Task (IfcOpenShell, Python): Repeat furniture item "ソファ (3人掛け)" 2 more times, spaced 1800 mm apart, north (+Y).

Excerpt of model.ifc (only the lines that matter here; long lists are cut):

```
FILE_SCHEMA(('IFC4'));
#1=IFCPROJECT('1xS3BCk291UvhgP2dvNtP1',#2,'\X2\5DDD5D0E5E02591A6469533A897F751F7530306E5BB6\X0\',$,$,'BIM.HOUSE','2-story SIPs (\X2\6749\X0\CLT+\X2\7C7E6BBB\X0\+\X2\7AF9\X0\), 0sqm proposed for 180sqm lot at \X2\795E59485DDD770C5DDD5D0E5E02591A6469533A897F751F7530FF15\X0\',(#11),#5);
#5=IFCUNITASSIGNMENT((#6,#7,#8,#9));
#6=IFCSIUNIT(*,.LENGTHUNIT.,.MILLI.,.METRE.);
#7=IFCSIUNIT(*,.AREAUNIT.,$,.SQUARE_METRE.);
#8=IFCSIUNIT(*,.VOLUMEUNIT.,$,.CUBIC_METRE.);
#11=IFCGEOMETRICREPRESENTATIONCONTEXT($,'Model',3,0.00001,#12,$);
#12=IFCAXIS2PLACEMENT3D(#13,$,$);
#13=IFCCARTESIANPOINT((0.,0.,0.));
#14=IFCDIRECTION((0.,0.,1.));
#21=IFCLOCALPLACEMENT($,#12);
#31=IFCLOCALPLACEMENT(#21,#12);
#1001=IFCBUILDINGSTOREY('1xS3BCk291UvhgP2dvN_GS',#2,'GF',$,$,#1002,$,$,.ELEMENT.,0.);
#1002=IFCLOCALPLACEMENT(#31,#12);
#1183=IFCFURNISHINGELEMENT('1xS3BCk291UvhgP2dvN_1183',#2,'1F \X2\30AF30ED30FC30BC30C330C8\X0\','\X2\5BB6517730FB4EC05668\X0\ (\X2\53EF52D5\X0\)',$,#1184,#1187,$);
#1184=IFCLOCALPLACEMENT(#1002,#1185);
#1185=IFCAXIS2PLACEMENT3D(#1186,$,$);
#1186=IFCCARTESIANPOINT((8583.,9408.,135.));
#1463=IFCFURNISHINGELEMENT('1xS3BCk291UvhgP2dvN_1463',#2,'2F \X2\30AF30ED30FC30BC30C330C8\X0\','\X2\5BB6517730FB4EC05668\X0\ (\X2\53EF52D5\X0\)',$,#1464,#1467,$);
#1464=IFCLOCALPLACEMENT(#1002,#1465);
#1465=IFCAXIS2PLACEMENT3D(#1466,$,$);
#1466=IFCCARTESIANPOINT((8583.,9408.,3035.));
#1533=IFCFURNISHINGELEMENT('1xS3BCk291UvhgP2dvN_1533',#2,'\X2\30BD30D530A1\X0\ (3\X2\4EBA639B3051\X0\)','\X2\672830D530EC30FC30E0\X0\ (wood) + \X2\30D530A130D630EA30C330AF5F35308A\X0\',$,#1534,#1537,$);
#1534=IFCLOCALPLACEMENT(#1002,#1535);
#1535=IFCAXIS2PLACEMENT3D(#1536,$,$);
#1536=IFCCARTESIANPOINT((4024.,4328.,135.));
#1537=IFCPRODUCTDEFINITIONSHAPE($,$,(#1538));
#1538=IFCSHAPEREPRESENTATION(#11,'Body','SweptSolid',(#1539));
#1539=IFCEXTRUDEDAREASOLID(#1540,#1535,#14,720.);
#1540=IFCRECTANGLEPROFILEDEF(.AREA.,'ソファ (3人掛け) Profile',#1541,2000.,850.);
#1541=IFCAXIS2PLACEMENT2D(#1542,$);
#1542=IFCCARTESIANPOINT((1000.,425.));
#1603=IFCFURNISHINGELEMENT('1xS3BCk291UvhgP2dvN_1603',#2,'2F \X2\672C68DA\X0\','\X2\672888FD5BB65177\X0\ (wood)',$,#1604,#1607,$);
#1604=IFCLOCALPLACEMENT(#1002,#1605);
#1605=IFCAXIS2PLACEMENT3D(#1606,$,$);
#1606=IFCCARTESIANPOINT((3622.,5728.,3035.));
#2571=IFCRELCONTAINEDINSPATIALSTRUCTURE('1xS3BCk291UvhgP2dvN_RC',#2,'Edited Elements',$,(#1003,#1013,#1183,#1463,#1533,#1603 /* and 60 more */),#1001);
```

```python
import numpy as np
import ifcopenshell
import ifcopenshell.api.geometry
import ifcopenshell.api.root
import ifcopenshell.util.element
import ifcopenshell.util.placement
import ifcopenshell.util.unit

model = ifcopenshell.open("model.ifc")
unit_scale = ifcopenshell.util.unit.calculate_unit_scale(model)


def reuse_history(source, copy):
    """copy_class also copies each property set's owner history, people and application; keep the originals."""
    for rel in copy.IsDefinedBy:
        if rel.is_a("IfcRelDefinesByProperties") and (history := rel.RelatingPropertyDefinition.OwnerHistory):
            rel.RelatingPropertyDefinition.OwnerHistory = source.OwnerHistory
            ifcopenshell.util.element.remove_deep2(model, history)


source = model.by_guid("1xS3BCk291UvhgP2dvN_1533")
base = ifcopenshell.util.placement.get_local_placement(source.ObjectPlacement)
step = np.array([0.0, 1.0, 0.0]) * 1.8 / unit_scale

for i in range(1, 3):
    copy = ifcopenshell.api.root.copy_class(model, product=source)
    copy.Representation = ifcopenshell.util.element.copy_deep(
        model, source.Representation, exclude=["IfcGeometricRepresentationContext", "IfcRepresentationMap"]
    )
    reuse_history(source, copy)
    matrix = base.copy()
    matrix[:3, 3] += i * step
    print("added at", matrix[:3, 3].round(3) + 0.0)
    ifcopenshell.api.geometry.edit_object_placement(model, product=copy, matrix=matrix, is_si=False)

model.write("model_v2.ifc")
```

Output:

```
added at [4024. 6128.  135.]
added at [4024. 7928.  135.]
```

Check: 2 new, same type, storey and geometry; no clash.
